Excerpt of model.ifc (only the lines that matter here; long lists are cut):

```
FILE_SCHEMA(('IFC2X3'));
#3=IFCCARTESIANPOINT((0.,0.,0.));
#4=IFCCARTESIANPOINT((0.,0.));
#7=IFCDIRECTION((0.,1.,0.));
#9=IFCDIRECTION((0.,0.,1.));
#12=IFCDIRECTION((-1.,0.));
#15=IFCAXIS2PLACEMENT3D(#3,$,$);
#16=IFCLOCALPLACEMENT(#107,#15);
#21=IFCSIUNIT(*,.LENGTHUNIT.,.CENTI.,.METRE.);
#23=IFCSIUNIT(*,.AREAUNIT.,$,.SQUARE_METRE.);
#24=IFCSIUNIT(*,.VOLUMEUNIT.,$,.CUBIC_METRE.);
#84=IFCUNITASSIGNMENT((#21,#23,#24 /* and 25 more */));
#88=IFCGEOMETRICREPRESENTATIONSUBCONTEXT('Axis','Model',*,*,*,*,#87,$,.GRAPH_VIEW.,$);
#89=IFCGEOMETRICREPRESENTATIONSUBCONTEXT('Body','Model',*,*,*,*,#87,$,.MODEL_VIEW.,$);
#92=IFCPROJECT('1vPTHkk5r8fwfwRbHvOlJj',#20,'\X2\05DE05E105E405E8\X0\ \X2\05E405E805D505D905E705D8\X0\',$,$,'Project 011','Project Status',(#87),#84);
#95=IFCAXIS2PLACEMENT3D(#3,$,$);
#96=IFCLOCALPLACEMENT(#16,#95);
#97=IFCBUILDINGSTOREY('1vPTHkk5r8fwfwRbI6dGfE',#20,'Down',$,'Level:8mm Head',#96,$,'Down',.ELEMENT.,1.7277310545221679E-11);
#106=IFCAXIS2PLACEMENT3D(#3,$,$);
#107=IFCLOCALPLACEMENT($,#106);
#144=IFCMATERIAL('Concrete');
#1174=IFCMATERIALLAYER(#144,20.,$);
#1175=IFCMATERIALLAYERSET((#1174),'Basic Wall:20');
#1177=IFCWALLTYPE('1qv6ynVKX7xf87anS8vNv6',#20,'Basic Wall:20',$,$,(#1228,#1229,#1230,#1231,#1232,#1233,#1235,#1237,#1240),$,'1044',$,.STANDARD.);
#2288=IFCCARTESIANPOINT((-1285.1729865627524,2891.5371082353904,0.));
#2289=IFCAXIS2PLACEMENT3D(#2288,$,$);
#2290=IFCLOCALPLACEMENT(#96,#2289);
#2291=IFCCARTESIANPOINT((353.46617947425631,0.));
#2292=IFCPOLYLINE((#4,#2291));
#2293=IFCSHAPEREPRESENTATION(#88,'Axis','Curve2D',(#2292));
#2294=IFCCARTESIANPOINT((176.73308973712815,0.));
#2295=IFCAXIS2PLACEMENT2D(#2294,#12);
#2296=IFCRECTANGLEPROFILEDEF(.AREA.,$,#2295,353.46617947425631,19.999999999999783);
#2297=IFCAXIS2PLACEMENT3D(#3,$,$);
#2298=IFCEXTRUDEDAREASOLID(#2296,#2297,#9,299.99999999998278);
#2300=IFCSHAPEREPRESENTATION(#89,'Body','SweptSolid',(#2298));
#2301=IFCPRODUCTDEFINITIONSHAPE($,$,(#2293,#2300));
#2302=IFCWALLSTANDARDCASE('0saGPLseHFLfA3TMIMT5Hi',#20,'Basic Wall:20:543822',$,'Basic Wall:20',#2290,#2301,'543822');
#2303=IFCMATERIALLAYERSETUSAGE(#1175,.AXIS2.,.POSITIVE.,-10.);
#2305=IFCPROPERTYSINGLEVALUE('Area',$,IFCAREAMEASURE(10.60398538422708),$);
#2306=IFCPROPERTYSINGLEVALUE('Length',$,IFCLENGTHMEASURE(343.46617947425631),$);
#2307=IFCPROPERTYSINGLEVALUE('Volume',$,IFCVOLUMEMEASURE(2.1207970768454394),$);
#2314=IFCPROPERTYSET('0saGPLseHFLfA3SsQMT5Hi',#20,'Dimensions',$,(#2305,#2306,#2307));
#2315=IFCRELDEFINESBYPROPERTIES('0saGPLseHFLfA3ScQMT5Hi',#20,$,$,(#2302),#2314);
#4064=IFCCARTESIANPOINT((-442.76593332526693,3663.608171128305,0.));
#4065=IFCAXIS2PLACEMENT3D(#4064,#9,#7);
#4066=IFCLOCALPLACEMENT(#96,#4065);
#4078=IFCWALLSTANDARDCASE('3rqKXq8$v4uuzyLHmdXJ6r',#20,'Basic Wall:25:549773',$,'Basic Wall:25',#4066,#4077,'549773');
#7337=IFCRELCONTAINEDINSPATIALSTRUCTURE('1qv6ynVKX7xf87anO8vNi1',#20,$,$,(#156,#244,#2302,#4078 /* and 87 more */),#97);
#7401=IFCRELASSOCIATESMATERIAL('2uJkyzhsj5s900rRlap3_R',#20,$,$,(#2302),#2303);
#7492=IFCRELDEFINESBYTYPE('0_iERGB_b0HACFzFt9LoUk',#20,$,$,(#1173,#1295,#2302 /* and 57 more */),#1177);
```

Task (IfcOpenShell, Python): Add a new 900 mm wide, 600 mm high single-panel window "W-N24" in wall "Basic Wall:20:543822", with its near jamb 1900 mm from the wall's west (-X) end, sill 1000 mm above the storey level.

```python
import numpy as np
import ifcopenshell
import ifcopenshell.api.feature
import ifcopenshell.api.geometry
import ifcopenshell.api.pset
import ifcopenshell.api.root
import ifcopenshell.api.spatial
import ifcopenshell.api.type
import ifcopenshell.geom
import ifcopenshell.util.element
import ifcopenshell.util.placement
import ifcopenshell.util.representation
import ifcopenshell.util.shape
import ifcopenshell.util.unit

model = ifcopenshell.open("model.ifc")
unit_scale = ifcopenshell.util.unit.calculate_unit_scale(model)
area_scale = ifcopenshell.util.unit.calculate_unit_scale(model, "AREAUNIT")
volume_scale = ifcopenshell.util.unit.calculate_unit_scale(model, "VOLUMEUNIT")
settings = ifcopenshell.geom.settings()


def volume(element):
    """Net volume in cubic metres, openings subtracted."""
    shape = ifcopenshell.geom.create_shape(settings, element)
    return ifcopenshell.util.shape.get_volume(shape.geometry)


wall = model.by_id(2302)
storey = ifcopenshell.util.element.get_container(wall, ifc_class="IfcBuildingStorey")
context = ifcopenshell.util.representation.get_context(model, "Model", "Body", "MODEL_VIEW")
before = volume(wall)

width, height, from_end, sill = 0.9, 0.6, 1.9, 1  # metres

# The wall runs along its own X axis, and the end named is its -X end.
wall_shape = ifcopenshell.geom.create_shape(settings, wall)
x, y, z = ifcopenshell.util.shape.get_vertices(wall_shape.geometry).T
start = x.min() + from_end
face, thickness = float(y.min()), float(y.max() - y.min())
wall_matrix = ifcopenshell.util.placement.get_local_placement(wall.ObjectPlacement)
level = ifcopenshell.util.placement.get_local_placement(storey.ObjectPlacement)[2, 3]


def in_wall(x, y):
    """Placement at x, y metres in the wall's axes, at sill height."""
    matrix = wall_matrix.copy()
    matrix[:, 3] = wall_matrix @ np.array([x / unit_scale, y / unit_scale, 0.0, 1.0])
    matrix[2, 3] = level + sill / unit_scale
    return matrix


# Opening: a box that overshoots both wall faces by 50 mm.
opening = ifcopenshell.api.root.create_entity(model, ifc_class="IfcOpeningElement")
box = ifcopenshell.api.geometry.add_wall_representation(
    model, context=context, length=width, height=height, thickness=thickness + 0.1
)
ifcopenshell.api.geometry.assign_representation(model, product=opening, representation=box)
ifcopenshell.api.geometry.edit_object_placement(model, product=opening, matrix=in_wall(start, face - 0.05), is_si=False)
ifcopenshell.api.feature.add_feature(model, feature=opening, element=wall)

window = ifcopenshell.api.root.create_entity(model, ifc_class="IfcWindow", name="W-N24")
window.OverallWidth, window.OverallHeight = width / unit_scale, height / unit_scale
body = ifcopenshell.api.geometry.add_window_representation(
    model,
    context=context,
    overall_width=window.OverallWidth,
    overall_height=window.OverallHeight,
    partition_type="SINGLE_PANEL",
)
ifcopenshell.api.geometry.assign_representation(model, product=window, representation=body)
ifcopenshell.api.spatial.assign_container(model, products=[window], relating_structure=storey)
fills = ifcopenshell.api.feature.add_filling(model, opening=opening, element=window)
fills.OwnerHistory = window.OwnerHistory  # required in IFC2X3

# IFC2X3 keeps the operation on the window style.
style = ifcopenshell.api.root.create_entity(model, ifc_class="IfcWindowStyle", name="W-N24")
style.OperationType, style.ConstructionType = "SINGLE_PANEL", "NOTDEFINED"
style.ParameterTakesPrecedence = style.Sizeable = False
ifcopenshell.api.type.assign_type(model, related_objects=[window], relating_type=style)

# Centre the window in the wall's thickness.
ifcopenshell.api.geometry.edit_object_placement(model, product=window, matrix=in_wall(start, face), is_si=False)
window_shape = ifcopenshell.geom.create_shape(settings, window)
depth = ifcopenshell.util.shape.get_vertices(window_shape.geometry)[:, 1]
offset = face + thickness / 2 - (depth.min() + depth.max()) / 2
ifcopenshell.api.geometry.edit_object_placement(model, product=window, matrix=in_wall(start, offset), is_si=False)

after = volume(wall)

# Update the wall's stored quantities.
pset = model.by_id(ifcopenshell.util.element.get_pset(wall, "Dimensions", should_inherit=False)["id"])
ifcopenshell.api.pset.edit_pset(model, pset=pset, properties={
    "Area": model.create_entity("IfcAreaMeasure", after / thickness / area_scale),
    "Volume": model.create_entity("IfcVolumeMeasure", after / volume_scale),
})

print(f"wall volume {before:.3f} -> {after:.3f} m3")

model.write("model_edited.ifc")
```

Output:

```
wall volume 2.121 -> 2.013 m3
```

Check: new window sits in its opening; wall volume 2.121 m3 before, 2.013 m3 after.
